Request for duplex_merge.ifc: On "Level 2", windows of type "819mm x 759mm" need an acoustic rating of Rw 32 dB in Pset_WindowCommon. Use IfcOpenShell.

First a look at what the model holds.

```python
import ifcopenshell
import ifcopenshell.util.element

model = ifcopenshell.open("duplex_merge.ifc")
print(model.schema)
storey = next(s for s in model.by_type("IfcBuildingStorey") if s.Name == "Level 2")
windows = [e for e in ifcopenshell.util.element.get_decomposition(storey) if e.is_a("IfcWindow")]
seen = {}
for e in windows:
    element_type = ifcopenshell.util.element.get_type(e)
    key = (element_type.Name if element_type != e and element_type else None, ifcopenshell.util.element.get_pset(e, "Pset_WindowCommon", "AcousticRating"))
    seen[key] = seen.get(key, 0) + 1
for (name, value), count in sorted(seen.items(), key=str):
    print(count, "x", name, "|", value)
```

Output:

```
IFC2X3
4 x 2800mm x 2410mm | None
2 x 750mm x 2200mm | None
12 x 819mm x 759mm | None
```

```python
import ifcopenshell
import ifcopenshell.api.pset
import ifcopenshell.util.element

model = ifcopenshell.open("duplex_merge.ifc")

storey = next(s for s in model.by_type("IfcBuildingStorey") if s.Name == "Level 2")
windows = [e for e in ifcopenshell.util.element.get_decomposition(storey) if e.is_a("IfcWindow")]

count = 0
for e in windows:
    element_type = ifcopenshell.util.element.get_type(e)
    if element_type in (None, e) or element_type.Name != "819mm x 759mm":
        continue
    # add_pset returns the element's existing set when there is one.
    pset = ifcopenshell.api.pset.add_pset(model, product=e, name="Pset_WindowCommon")
    ifcopenshell.api.pset.edit_pset(model, pset=pset, properties={"AcousticRating": "Rw 32 dB"})
    count += 1

print(count, "windows updated")

model.write("duplex_merge_rev.ifc")
```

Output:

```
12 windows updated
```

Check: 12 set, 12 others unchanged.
